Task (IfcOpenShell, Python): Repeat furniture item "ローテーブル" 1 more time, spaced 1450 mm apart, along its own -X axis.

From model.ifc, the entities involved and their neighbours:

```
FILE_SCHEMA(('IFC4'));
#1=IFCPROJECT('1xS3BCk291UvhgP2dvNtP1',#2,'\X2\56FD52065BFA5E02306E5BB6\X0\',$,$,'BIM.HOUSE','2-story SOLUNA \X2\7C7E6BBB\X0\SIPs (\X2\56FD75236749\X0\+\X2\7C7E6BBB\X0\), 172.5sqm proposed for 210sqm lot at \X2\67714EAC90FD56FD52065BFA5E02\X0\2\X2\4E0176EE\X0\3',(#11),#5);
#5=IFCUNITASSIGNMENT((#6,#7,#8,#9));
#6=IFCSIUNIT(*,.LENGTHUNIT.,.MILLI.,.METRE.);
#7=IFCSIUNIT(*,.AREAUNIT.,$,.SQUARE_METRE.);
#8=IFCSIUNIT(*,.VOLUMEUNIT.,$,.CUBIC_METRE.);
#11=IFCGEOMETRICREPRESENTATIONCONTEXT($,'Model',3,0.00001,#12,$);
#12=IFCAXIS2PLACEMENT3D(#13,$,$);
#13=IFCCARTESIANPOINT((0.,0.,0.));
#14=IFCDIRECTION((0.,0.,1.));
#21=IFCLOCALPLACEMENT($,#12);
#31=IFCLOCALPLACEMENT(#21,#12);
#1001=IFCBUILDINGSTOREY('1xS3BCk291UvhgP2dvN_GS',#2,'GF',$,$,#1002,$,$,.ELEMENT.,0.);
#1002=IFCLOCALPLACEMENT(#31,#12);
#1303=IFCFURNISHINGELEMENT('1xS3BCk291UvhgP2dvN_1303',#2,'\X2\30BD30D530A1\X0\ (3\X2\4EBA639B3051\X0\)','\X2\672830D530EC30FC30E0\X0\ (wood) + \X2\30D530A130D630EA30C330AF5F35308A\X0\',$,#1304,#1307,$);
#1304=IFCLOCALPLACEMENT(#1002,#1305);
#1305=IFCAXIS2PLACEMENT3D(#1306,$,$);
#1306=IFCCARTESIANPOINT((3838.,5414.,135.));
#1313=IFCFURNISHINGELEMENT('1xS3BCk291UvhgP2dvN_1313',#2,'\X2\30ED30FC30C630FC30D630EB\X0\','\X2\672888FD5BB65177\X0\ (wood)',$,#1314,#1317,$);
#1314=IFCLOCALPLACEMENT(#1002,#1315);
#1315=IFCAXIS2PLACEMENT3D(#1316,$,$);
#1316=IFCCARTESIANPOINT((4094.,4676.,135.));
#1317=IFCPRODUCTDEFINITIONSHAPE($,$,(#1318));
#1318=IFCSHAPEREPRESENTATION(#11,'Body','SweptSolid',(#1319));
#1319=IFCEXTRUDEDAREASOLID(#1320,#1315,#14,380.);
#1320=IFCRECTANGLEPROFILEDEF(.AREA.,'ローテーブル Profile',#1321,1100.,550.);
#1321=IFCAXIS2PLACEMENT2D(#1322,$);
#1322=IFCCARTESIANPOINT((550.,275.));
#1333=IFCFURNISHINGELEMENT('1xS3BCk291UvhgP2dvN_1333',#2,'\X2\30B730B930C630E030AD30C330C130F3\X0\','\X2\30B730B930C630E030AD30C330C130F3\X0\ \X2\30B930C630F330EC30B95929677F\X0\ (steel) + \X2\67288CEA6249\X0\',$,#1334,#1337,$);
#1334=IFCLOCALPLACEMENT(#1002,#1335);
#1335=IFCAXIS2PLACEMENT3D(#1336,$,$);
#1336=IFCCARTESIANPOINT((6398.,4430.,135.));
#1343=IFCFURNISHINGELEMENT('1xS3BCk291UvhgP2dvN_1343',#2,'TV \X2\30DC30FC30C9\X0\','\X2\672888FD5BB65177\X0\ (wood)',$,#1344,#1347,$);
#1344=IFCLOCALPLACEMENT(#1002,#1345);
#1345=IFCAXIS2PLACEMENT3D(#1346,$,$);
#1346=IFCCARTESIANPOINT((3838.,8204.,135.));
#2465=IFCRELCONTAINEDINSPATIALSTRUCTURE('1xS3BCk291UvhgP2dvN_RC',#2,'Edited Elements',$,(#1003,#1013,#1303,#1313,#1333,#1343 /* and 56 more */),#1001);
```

```python
import ifcopenshell
import ifcopenshell.api.geometry
import ifcopenshell.api.root
import ifcopenshell.util.element
import ifcopenshell.util.placement
import ifcopenshell.util.unit

model = ifcopenshell.open("model.ifc")
unit_scale = ifcopenshell.util.unit.calculate_unit_scale(model)


def reuse_history(source, copy):
    """copy_class also copies each property set's owner history, people and application; keep the originals."""
    for rel in copy.IsDefinedBy:
        if rel.is_a("IfcRelDefinesByProperties") and (history := rel.RelatingPropertyDefinition.OwnerHistory):
            rel.RelatingPropertyDefinition.OwnerHistory = source.OwnerHistory
            ifcopenshell.util.element.remove_deep2(model, history)


source = model.by_guid("1xS3BCk291UvhgP2dvN_1313")
base = ifcopenshell.util.placement.get_local_placement(source.ObjectPlacement)
step = -base[:3, 0] * 1.45 / unit_scale

for i in range(1, 2):
    copy = ifcopenshell.api.root.copy_class(model, product=source)
    copy.Representation = ifcopenshell.util.element.copy_deep(
        model, source.Representation, exclude=["IfcGeometricRepresentationContext", "IfcRepresentationMap"]
    )
    reuse_history(source, copy)
    matrix = base.copy()
    matrix[:3, 3] += i * step
    print("added at", matrix[:3, 3].round(3) + 0.0)
    ifcopenshell.api.geometry.edit_object_placement(model, product=copy, matrix=matrix, is_si=False)

model.write("model_updated.ifc")
```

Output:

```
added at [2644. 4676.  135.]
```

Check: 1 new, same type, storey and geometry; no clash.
